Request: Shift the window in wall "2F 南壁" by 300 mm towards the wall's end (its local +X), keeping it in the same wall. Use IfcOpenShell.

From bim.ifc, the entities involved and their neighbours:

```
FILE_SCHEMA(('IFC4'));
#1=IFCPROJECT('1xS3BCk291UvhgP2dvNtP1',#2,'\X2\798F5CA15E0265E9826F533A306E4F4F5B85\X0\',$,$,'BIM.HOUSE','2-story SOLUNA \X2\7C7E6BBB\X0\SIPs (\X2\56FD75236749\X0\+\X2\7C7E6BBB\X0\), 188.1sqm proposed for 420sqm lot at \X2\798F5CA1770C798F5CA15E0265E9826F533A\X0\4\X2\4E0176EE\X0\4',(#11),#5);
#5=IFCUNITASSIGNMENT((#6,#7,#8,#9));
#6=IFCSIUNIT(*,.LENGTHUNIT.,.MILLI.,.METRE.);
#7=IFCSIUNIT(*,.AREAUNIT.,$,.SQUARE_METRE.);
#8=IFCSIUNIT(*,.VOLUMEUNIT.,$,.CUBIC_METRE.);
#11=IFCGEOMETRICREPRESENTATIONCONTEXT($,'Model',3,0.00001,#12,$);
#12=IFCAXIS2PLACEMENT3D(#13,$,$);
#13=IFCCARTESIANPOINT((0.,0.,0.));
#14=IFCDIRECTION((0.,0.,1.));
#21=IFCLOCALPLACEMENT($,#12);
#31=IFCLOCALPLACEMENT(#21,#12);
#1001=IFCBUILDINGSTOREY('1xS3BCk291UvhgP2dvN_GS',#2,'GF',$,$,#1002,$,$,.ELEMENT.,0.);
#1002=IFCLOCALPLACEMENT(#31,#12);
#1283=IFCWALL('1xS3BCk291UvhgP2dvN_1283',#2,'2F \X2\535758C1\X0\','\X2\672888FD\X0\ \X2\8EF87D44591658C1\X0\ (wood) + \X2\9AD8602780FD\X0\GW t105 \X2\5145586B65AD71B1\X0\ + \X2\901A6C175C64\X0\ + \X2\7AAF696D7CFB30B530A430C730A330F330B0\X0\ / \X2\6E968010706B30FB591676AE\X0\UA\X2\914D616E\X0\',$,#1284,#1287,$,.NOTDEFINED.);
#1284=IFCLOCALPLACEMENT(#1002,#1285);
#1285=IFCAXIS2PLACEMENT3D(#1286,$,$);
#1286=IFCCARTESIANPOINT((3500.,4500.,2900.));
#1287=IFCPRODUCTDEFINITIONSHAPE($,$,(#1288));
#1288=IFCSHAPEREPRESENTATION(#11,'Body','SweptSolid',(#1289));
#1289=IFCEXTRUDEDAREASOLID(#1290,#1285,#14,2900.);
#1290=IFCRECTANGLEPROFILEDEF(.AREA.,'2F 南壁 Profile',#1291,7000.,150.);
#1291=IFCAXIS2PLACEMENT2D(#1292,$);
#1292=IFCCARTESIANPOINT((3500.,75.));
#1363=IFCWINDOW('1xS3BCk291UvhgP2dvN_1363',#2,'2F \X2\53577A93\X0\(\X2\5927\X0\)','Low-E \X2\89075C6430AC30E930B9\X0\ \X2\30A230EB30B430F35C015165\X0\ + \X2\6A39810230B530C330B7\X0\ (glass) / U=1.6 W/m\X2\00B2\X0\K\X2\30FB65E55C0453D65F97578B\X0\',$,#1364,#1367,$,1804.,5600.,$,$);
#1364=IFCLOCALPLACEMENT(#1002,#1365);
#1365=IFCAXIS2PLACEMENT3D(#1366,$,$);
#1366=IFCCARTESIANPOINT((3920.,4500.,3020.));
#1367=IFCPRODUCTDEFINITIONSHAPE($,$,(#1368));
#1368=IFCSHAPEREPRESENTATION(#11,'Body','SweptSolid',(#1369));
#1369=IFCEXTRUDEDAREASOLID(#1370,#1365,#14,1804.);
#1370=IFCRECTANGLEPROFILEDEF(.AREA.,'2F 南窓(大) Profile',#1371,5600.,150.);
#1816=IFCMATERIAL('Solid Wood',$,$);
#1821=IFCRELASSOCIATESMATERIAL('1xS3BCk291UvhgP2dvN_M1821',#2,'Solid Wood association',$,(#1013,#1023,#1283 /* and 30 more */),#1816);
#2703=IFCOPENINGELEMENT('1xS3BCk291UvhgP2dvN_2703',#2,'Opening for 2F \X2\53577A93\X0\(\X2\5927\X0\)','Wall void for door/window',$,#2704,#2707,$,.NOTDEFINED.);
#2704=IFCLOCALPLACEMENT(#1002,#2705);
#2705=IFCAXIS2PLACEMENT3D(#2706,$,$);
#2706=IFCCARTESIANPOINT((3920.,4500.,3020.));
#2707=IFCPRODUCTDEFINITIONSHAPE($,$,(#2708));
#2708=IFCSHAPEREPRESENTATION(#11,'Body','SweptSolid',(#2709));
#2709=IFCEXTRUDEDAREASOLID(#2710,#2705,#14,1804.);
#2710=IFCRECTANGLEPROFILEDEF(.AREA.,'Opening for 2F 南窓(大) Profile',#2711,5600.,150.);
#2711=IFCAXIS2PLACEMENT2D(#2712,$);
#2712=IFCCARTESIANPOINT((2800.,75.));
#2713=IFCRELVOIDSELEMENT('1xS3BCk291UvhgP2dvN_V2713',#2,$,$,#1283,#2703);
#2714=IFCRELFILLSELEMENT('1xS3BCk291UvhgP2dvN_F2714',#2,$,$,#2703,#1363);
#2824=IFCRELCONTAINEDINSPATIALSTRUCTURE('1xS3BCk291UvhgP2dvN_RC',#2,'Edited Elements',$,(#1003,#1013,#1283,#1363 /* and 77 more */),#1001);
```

```python
import ifcopenshell
import ifcopenshell.api.geometry
import ifcopenshell.util.placement
import ifcopenshell.util.unit

model = ifcopenshell.open("bim.ifc")
unit_scale = ifcopenshell.util.unit.calculate_unit_scale(model)

window = model.by_guid("1xS3BCk291UvhgP2dvN_1363")
opening = window.FillsVoids[0].RelatingOpeningElement
wall = opening.VoidsElements[0].RelatingBuildingElement

wall_matrix = ifcopenshell.util.placement.get_local_placement(wall.ObjectPlacement)
shift = wall_matrix[:3, 0] * 0.3 / unit_scale
before = ifcopenshell.util.placement.get_local_placement(window.ObjectPlacement)[:3, 3].copy()

# The window is not placed relative to its opening, so move both.
for product in (opening, window):
    matrix = ifcopenshell.util.placement.get_local_placement(product.ObjectPlacement)
    matrix[:3, 3] += shift
    ifcopenshell.api.geometry.edit_object_placement(model, product=product, matrix=matrix, is_si=False)

after = ifcopenshell.util.placement.get_local_placement(window.ObjectPlacement)[:3, 3]
print("window moved by", (after - before).round(3) + 0.0)

model.write("bim_rev.ifc")
```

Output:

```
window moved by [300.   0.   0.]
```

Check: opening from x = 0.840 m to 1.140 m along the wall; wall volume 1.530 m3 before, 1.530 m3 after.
